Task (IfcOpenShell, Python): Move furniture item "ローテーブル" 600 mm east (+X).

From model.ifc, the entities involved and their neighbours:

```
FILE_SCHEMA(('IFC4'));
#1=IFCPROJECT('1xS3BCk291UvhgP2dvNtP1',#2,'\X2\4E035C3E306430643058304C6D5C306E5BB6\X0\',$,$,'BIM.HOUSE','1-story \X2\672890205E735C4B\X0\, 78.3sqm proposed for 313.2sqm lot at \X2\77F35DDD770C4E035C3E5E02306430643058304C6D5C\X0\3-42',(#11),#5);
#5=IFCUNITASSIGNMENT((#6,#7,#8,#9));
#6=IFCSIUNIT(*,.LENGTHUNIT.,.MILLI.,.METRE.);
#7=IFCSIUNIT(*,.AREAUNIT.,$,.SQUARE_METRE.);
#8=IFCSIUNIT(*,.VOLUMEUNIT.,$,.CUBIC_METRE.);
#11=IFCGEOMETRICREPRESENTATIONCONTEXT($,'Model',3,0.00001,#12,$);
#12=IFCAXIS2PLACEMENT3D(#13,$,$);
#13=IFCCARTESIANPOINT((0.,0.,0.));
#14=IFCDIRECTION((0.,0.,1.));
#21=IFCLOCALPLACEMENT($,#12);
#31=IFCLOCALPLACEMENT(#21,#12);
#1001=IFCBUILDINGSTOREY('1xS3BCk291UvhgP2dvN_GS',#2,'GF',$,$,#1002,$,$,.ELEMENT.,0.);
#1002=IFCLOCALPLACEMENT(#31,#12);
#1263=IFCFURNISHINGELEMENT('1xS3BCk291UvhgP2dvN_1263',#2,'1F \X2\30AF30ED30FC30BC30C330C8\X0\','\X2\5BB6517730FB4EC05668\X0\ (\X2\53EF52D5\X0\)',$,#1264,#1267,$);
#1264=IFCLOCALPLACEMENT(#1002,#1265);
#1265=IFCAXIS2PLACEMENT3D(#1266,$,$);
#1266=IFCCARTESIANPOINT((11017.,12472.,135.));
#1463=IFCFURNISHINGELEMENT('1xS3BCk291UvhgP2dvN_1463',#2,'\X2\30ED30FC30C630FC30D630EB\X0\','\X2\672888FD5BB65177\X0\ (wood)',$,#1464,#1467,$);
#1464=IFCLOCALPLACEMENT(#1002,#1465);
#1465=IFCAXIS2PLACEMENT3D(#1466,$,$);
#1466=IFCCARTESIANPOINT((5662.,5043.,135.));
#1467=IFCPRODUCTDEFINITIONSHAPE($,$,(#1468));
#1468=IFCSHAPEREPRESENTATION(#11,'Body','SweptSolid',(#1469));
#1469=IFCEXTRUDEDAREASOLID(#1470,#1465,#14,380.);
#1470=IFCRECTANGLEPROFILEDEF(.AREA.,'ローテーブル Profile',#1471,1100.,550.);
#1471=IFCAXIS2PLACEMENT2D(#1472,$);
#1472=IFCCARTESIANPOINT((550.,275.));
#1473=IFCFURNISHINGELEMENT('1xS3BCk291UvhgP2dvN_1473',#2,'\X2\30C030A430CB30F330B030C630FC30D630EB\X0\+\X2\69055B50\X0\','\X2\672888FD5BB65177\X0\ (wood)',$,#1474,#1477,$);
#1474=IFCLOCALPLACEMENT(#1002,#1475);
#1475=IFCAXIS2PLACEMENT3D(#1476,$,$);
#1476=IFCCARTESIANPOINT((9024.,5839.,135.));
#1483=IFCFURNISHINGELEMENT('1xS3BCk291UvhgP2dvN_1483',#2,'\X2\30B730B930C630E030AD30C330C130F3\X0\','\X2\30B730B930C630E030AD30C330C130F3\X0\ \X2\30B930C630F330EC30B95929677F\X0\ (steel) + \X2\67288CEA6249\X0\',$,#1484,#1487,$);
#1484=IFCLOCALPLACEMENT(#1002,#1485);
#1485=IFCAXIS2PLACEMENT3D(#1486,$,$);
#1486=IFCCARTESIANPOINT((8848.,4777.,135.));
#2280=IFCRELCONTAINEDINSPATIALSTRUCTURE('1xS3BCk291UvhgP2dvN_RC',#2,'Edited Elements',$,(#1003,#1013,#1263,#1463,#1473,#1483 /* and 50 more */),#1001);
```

```python
import ifcopenshell
import ifcopenshell.api.geometry
import ifcopenshell.util.placement
import ifcopenshell.util.unit

model = ifcopenshell.open("model.ifc")
unit_scale = ifcopenshell.util.unit.calculate_unit_scale(model)

item = model.by_id(1463)
matrix = ifcopenshell.util.placement.get_local_placement(item.ObjectPlacement)
matrix[0, 3] += 0.6 / unit_scale
ifcopenshell.api.geometry.edit_object_placement(model, product=item, matrix=matrix, is_si=False)

print(ifcopenshell.util.placement.get_local_placement(item.ObjectPlacement).round(3) + 0.0)

model.write("model-out.ifc")
```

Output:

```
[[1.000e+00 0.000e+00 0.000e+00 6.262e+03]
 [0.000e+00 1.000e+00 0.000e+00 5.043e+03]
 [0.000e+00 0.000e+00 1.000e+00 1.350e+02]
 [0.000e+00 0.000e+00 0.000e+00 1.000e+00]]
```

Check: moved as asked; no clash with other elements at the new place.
